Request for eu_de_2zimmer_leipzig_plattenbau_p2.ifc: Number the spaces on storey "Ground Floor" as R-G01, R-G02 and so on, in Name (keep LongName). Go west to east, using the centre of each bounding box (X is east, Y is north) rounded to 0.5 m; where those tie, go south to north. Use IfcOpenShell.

First a look at what the model holds.

```python
import ifcopenshell
import ifcopenshell.util.element
import ifcopenshell.util.placement

model = ifcopenshell.open("eu_de_2zimmer_leipzig_plattenbau_p2.ifc")
print(model.schema)
storey = next(s for s in model.by_type("IfcBuildingStorey") if s.Name == "Ground Floor")
spaces = [e for e in ifcopenshell.util.element.get_decomposition(storey) if e.is_a("IfcSpace")]
for e in sorted(spaces, key=lambda e: e.id()):
    origin = ifcopenshell.util.placement.get_local_placement(e.ObjectPlacement)[:3, 3]
    print(e.id(), e.Name, e.LongName, origin.round(2) + 0.0, sep=" | ")
```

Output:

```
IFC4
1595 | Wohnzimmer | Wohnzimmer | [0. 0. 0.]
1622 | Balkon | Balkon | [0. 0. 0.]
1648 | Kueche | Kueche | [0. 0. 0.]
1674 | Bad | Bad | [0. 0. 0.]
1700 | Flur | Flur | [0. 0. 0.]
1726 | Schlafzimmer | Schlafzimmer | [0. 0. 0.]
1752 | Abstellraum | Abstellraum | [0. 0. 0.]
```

```python
import ifcopenshell
import ifcopenshell.geom
import ifcopenshell.util.element
import ifcopenshell.util.shape

model = ifcopenshell.open("eu_de_2zimmer_leipzig_plattenbau_p2.ifc")
settings = ifcopenshell.geom.settings()
settings.set("use-world-coords", True)


def centre(element):
    shape = ifcopenshell.geom.create_shape(settings, element)
    return ifcopenshell.util.shape.get_bbox_centroid(shape.geometry)


storey = next(s for s in model.by_type("IfcBuildingStorey") if s.Name == "Ground Floor")
spaces = [e for e in ifcopenshell.util.element.get_decomposition(storey) if e.is_a("IfcSpace")]

# Insertion points can sit at a corner or the storey origin, so sort by the geometry (in metres).
centres = {e: centre(e) for e in spaces}
spaces.sort(key=lambda e: (round(centres[e][0] / 0.5), centres[e][1]))

for i, e in enumerate(spaces, start=1):
    number = f"R-G{i:02d}"
    e.Name = number
    print(e.id(), number)

model.write("eu_de_2zimmer_leipzig_plattenbau_p2_edited.ifc")
```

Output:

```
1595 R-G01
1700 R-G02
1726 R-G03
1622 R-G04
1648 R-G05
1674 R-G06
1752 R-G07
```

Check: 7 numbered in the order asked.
